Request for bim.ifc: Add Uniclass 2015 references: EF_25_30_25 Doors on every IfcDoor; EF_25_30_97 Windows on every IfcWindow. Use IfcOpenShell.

First a look at what the model holds.

```python
import ifcopenshell

model = ifcopenshell.open("bim.ifc")
print(model.schema)
print("classifications:", [c.Name for c in model.by_type("IfcClassification")])
for ifc_class in ("IfcDoor", "IfcRoof", "IfcStair", "IfcWall", "IfcWindow"):
    print(ifc_class, len(model.by_type(ifc_class)))
```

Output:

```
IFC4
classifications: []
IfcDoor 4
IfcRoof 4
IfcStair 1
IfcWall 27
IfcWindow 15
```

```python
import ifcopenshell
import ifcopenshell.api.classification

model = ifcopenshell.open("bim.ifc")

system = ifcopenshell.api.classification.add_classification(model, classification="Uniclass 2015")

codes = {
    "IfcDoor": ("EF_25_30_25", "Doors"),
    "IfcWindow": ("EF_25_30_97", "Windows"),
}
for ifc_class, (code, name) in codes.items():
    products = model.by_type(ifc_class)
    ifcopenshell.api.classification.add_reference(
        model, products=products, classification=system, identification=code, name=name
    )
    print(code, len(products))

model.write("bim_v2.ifc")
```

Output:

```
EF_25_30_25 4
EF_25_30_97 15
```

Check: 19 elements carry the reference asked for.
